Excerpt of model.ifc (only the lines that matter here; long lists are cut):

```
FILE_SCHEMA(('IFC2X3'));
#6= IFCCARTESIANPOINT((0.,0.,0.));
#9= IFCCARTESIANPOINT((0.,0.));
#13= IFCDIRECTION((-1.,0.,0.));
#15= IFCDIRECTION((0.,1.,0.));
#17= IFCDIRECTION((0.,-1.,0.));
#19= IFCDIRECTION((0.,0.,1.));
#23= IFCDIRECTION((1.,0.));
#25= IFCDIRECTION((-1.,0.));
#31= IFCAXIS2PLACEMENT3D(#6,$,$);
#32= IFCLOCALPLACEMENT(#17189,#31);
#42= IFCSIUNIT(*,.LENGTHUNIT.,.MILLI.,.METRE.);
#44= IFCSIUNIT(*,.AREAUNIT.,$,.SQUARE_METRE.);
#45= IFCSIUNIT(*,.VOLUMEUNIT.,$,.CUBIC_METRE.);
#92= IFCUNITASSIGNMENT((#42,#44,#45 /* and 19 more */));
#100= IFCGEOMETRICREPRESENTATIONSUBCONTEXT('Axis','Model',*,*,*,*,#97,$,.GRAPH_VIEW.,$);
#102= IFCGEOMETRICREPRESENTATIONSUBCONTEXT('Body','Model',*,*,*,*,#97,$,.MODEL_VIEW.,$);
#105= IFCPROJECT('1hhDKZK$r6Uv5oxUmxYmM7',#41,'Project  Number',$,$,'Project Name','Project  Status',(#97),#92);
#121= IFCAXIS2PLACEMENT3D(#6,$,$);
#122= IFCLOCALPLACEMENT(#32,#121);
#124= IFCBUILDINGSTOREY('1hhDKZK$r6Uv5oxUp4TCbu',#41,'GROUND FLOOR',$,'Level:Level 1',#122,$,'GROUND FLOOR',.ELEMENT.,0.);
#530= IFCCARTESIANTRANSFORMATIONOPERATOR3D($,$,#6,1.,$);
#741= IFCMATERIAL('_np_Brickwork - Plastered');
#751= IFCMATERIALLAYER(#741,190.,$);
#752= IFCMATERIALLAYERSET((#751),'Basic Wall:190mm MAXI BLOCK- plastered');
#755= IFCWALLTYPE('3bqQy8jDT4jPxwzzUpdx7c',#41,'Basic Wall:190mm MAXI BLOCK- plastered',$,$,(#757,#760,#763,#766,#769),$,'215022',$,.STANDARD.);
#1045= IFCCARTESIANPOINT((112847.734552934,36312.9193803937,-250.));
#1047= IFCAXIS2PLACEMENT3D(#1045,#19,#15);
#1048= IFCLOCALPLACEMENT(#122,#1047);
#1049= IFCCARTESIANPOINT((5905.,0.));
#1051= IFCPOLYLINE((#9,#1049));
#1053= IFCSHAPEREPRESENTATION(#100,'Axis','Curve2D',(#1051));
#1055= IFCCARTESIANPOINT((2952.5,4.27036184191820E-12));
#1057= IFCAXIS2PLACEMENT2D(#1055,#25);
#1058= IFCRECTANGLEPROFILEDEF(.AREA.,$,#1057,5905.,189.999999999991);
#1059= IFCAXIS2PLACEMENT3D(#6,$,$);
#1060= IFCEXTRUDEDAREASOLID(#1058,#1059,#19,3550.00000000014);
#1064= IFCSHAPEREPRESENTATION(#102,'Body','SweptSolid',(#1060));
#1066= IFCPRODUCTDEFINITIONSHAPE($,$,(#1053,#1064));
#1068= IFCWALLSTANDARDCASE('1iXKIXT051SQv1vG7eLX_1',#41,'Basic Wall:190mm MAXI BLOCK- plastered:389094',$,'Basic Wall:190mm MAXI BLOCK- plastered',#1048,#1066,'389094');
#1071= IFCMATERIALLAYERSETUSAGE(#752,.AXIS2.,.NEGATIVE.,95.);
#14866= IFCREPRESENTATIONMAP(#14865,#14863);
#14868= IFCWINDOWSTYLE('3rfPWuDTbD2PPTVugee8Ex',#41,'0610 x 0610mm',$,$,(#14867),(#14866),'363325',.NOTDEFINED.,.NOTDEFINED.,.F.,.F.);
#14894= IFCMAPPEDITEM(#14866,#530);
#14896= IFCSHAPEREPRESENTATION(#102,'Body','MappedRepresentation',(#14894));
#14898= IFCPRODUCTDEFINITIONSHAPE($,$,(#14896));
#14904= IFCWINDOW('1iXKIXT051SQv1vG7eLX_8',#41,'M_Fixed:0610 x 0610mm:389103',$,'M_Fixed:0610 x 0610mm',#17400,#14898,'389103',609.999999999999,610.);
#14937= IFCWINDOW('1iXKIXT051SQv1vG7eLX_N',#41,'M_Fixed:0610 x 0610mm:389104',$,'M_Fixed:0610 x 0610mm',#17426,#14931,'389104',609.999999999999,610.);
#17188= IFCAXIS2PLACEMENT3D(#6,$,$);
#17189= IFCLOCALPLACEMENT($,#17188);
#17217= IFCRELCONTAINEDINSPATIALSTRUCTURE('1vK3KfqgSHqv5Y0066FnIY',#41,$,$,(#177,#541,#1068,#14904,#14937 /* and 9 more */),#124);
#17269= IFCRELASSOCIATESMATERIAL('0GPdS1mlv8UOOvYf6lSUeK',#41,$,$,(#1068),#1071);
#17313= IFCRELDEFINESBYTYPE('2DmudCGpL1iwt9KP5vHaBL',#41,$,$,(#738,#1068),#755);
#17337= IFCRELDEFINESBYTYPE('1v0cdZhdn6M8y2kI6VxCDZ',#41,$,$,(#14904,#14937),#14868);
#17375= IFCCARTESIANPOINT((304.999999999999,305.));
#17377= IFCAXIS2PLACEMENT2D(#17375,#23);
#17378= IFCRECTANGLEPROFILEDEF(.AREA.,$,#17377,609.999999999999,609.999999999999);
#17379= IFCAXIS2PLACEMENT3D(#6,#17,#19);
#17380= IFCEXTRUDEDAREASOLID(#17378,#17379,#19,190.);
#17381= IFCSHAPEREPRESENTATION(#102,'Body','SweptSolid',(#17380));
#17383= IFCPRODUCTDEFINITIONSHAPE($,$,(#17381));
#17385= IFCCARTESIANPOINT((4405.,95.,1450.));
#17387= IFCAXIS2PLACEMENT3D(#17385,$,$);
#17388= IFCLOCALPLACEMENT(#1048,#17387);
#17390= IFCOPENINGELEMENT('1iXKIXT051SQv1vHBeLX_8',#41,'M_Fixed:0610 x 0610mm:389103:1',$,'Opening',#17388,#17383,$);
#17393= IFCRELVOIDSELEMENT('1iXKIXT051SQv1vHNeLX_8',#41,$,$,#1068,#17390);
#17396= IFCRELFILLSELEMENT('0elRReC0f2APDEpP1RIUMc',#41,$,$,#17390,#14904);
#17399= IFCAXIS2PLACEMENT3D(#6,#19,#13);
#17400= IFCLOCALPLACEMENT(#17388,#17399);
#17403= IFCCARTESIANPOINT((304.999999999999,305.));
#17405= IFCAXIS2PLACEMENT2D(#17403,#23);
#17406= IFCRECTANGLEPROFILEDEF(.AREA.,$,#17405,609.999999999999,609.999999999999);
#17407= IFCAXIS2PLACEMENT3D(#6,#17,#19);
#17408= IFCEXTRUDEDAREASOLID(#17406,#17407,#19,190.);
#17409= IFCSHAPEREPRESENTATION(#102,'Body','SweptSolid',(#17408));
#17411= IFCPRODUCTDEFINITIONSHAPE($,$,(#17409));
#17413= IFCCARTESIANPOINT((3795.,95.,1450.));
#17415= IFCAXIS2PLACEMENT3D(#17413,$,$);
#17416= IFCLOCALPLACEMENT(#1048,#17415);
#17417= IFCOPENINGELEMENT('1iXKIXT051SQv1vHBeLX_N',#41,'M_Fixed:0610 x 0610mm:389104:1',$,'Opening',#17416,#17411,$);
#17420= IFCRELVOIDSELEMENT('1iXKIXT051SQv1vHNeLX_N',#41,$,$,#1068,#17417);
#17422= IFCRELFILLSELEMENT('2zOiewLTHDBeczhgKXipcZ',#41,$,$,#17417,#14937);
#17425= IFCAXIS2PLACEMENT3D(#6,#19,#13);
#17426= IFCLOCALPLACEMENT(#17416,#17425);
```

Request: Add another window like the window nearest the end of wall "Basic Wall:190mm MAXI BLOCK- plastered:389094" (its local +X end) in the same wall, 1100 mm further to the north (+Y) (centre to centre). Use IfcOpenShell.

```python
import ifcopenshell
import ifcopenshell.api.feature
import ifcopenshell.api.geometry
import ifcopenshell.api.root
import ifcopenshell.geom
import ifcopenshell.util.element
import ifcopenshell.util.placement
import ifcopenshell.util.shape

model = ifcopenshell.open("model.ifc")
settings = ifcopenshell.geom.settings()


def volume(element):
    """Net volume in cubic metres, openings subtracted."""
    shape = ifcopenshell.geom.create_shape(settings, element)
    return ifcopenshell.util.shape.get_volume(shape.geometry)


def reuse_history(source, copy):
    """copy_class also copies each property set's owner history, people and application; keep the originals."""
    for rel in copy.IsDefinedBy:
        if rel.is_a("IfcRelDefinesByProperties") and (history := rel.RelatingPropertyDefinition.OwnerHistory):
            rel.RelatingPropertyDefinition.OwnerHistory = source.OwnerHistory
            ifcopenshell.util.element.remove_deep2(model, history)


window = model.by_guid("1iXKIXT051SQv1vG7eLX_8")
opening = window.FillsVoids[0].RelatingOpeningElement
wall = opening.VoidsElements[0].RelatingBuildingElement
before = volume(wall)
shift = ifcopenshell.util.placement.get_local_placement(wall.ObjectPlacement)[:3, 0] * 1100.0

# copy_class copies the void relationship, type, container and properties, but no geometry.
new_opening = ifcopenshell.api.root.copy_class(model, product=opening)
new_opening.Representation = ifcopenshell.util.element.copy_deep(
    model, opening.Representation, exclude=["IfcGeometricRepresentationContext", "IfcRepresentationMap"]
)
new_opening.Name = "M_Fixed:0610 x 0610mm"
new_window = ifcopenshell.api.root.copy_class(model, product=window)
new_window.Representation = ifcopenshell.util.element.copy_deep(
    model, window.Representation, exclude=["IfcGeometricRepresentationContext", "IfcRepresentationMap"]
)
new_window.Name = "M_Fixed:0610 x 0610mm"
new_window.Tag = None
reuse_history(window, new_window)
fills = ifcopenshell.api.feature.add_filling(model, opening=new_opening, element=new_window)
fills.OwnerHistory = new_window.OwnerHistory  # required in IFC2X3

for old, new in ((opening, new_opening), (window, new_window)):
    matrix = ifcopenshell.util.placement.get_local_placement(old.ObjectPlacement)
    matrix[:3, 3] += shift
    ifcopenshell.api.geometry.edit_object_placement(model, product=new, matrix=matrix, is_si=False)

after = volume(wall)

print(f"wall volume {before:.3f} -> {after:.3f} m3")

model.write("model_rev.ifc")
```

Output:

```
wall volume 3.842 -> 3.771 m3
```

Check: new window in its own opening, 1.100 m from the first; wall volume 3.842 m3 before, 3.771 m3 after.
